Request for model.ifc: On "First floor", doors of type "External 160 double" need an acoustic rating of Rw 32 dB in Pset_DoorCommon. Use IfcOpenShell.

First a look at what the model holds.

```python
import ifcopenshell
import ifcopenshell.util.element

model = ifcopenshell.open("model.ifc")
print(model.schema)
storey = next(s for s in model.by_type("IfcBuildingStorey") if s.Name == "First floor")
doors = [e for e in ifcopenshell.util.element.get_decomposition(storey) if e.is_a("IfcDoor")]
seen = {}
for e in doors:
    element_type = ifcopenshell.util.element.get_type(e)
    key = (element_type.Name if element_type != e and element_type else None, ifcopenshell.util.element.get_pset(e, "Pset_DoorCommon", "AcousticRating"))
    seen[key] = seen.get(key, 0) + 1
for (name, value), count in sorted(seen.items(), key=str):
    print(count, "x", name, "|", value)
```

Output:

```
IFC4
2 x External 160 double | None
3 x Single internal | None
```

```python
import ifcopenshell
import ifcopenshell.api.pset
import ifcopenshell.util.element

model = ifcopenshell.open("model.ifc")

storey = next(s for s in model.by_type("IfcBuildingStorey") if s.Name == "First floor")
doors = [e for e in ifcopenshell.util.element.get_decomposition(storey) if e.is_a("IfcDoor")]

count = 0
for e in doors:
    element_type = ifcopenshell.util.element.get_type(e)
    if element_type in (None, e) or element_type.Name != "External 160 double":
        continue
    # add_pset returns the element's existing set when there is one.
    pset = ifcopenshell.api.pset.add_pset(model, product=e, name="Pset_DoorCommon")
    ifcopenshell.api.pset.edit_pset(model, pset=pset, properties={"AcousticRating": "Rw 32 dB"})
    count += 1

print(count, "doors updated")

model.write("model-out.ifc")
```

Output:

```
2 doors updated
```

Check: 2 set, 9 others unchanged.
